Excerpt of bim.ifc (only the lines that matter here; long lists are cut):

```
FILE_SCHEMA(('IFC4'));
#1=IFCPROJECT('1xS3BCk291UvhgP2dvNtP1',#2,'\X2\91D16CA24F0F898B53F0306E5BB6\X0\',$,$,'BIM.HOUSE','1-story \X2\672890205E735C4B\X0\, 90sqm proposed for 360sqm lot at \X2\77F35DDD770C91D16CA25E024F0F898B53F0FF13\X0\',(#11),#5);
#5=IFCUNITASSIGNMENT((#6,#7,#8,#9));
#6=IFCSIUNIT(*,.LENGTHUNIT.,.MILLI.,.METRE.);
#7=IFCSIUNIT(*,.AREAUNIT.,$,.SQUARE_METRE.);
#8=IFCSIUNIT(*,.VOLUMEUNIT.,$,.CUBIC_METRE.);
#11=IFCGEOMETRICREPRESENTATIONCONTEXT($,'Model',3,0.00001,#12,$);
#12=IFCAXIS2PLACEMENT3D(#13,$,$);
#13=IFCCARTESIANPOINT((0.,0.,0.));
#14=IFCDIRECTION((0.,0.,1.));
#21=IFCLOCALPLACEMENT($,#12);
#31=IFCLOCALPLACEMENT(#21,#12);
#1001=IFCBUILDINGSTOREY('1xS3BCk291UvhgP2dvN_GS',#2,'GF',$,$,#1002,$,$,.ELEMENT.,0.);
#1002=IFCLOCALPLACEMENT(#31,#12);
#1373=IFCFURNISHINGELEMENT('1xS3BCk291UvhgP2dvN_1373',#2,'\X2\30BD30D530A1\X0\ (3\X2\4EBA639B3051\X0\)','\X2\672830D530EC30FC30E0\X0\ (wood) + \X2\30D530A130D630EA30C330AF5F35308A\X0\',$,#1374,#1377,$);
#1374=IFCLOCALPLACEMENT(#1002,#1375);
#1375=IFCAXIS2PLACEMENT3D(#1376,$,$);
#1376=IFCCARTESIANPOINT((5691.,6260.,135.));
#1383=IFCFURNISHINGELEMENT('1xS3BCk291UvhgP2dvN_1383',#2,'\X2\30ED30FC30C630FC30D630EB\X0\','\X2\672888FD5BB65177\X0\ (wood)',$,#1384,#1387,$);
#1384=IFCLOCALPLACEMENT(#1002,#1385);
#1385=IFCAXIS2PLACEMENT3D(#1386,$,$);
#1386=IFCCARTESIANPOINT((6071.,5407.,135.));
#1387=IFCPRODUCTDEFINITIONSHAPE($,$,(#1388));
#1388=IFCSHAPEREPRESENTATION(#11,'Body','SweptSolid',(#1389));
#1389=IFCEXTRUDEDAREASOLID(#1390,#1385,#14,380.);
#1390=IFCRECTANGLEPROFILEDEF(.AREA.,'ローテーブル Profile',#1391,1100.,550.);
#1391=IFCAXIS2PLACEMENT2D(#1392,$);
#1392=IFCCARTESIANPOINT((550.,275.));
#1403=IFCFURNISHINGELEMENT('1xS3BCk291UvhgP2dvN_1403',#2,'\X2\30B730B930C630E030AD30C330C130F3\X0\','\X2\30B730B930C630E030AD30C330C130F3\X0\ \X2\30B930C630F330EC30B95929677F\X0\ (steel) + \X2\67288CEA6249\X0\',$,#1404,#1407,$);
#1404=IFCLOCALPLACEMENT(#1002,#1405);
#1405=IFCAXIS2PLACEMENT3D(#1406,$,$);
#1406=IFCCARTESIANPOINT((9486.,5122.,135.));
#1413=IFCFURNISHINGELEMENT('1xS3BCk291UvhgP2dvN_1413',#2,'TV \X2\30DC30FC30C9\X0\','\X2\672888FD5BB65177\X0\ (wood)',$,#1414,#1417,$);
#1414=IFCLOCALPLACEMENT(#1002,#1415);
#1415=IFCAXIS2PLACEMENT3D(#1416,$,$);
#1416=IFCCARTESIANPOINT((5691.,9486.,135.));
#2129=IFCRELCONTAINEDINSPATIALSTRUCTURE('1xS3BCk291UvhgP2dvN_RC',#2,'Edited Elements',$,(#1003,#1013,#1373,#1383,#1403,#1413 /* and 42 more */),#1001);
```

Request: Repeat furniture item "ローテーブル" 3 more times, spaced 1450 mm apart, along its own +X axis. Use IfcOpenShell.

```python
import ifcopenshell
import ifcopenshell.api.geometry
import ifcopenshell.api.root
import ifcopenshell.util.element
import ifcopenshell.util.placement
import ifcopenshell.util.unit

model = ifcopenshell.open("bim.ifc")
unit_scale = ifcopenshell.util.unit.calculate_unit_scale(model)


def reuse_history(source, copy):
    """copy_class also copies each property set's owner history, people and application; keep the originals."""
    for rel in copy.IsDefinedBy:
        if rel.is_a("IfcRelDefinesByProperties") and (history := rel.RelatingPropertyDefinition.OwnerHistory):
            rel.RelatingPropertyDefinition.OwnerHistory = source.OwnerHistory
            ifcopenshell.util.element.remove_deep2(model, history)


source = model.by_id(1383)
base = ifcopenshell.util.placement.get_local_placement(source.ObjectPlacement)
step = base[:3, 0] * 1.45 / unit_scale

for i in range(1, 4):
    copy = ifcopenshell.api.root.copy_class(model, product=source)
    copy.Representation = ifcopenshell.util.element.copy_deep(
        model, source.Representation, exclude=["IfcGeometricRepresentationContext", "IfcRepresentationMap"]
    )
    reuse_history(source, copy)
    matrix = base.copy()
    matrix[:3, 3] += i * step
    print("added at", matrix[:3, 3].round(3) + 0.0)
    ifcopenshell.api.geometry.edit_object_placement(model, product=copy, matrix=matrix, is_si=False)

model.write("bim_updated.ifc")
```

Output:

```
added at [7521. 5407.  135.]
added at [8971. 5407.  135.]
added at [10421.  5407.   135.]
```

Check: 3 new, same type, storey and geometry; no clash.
